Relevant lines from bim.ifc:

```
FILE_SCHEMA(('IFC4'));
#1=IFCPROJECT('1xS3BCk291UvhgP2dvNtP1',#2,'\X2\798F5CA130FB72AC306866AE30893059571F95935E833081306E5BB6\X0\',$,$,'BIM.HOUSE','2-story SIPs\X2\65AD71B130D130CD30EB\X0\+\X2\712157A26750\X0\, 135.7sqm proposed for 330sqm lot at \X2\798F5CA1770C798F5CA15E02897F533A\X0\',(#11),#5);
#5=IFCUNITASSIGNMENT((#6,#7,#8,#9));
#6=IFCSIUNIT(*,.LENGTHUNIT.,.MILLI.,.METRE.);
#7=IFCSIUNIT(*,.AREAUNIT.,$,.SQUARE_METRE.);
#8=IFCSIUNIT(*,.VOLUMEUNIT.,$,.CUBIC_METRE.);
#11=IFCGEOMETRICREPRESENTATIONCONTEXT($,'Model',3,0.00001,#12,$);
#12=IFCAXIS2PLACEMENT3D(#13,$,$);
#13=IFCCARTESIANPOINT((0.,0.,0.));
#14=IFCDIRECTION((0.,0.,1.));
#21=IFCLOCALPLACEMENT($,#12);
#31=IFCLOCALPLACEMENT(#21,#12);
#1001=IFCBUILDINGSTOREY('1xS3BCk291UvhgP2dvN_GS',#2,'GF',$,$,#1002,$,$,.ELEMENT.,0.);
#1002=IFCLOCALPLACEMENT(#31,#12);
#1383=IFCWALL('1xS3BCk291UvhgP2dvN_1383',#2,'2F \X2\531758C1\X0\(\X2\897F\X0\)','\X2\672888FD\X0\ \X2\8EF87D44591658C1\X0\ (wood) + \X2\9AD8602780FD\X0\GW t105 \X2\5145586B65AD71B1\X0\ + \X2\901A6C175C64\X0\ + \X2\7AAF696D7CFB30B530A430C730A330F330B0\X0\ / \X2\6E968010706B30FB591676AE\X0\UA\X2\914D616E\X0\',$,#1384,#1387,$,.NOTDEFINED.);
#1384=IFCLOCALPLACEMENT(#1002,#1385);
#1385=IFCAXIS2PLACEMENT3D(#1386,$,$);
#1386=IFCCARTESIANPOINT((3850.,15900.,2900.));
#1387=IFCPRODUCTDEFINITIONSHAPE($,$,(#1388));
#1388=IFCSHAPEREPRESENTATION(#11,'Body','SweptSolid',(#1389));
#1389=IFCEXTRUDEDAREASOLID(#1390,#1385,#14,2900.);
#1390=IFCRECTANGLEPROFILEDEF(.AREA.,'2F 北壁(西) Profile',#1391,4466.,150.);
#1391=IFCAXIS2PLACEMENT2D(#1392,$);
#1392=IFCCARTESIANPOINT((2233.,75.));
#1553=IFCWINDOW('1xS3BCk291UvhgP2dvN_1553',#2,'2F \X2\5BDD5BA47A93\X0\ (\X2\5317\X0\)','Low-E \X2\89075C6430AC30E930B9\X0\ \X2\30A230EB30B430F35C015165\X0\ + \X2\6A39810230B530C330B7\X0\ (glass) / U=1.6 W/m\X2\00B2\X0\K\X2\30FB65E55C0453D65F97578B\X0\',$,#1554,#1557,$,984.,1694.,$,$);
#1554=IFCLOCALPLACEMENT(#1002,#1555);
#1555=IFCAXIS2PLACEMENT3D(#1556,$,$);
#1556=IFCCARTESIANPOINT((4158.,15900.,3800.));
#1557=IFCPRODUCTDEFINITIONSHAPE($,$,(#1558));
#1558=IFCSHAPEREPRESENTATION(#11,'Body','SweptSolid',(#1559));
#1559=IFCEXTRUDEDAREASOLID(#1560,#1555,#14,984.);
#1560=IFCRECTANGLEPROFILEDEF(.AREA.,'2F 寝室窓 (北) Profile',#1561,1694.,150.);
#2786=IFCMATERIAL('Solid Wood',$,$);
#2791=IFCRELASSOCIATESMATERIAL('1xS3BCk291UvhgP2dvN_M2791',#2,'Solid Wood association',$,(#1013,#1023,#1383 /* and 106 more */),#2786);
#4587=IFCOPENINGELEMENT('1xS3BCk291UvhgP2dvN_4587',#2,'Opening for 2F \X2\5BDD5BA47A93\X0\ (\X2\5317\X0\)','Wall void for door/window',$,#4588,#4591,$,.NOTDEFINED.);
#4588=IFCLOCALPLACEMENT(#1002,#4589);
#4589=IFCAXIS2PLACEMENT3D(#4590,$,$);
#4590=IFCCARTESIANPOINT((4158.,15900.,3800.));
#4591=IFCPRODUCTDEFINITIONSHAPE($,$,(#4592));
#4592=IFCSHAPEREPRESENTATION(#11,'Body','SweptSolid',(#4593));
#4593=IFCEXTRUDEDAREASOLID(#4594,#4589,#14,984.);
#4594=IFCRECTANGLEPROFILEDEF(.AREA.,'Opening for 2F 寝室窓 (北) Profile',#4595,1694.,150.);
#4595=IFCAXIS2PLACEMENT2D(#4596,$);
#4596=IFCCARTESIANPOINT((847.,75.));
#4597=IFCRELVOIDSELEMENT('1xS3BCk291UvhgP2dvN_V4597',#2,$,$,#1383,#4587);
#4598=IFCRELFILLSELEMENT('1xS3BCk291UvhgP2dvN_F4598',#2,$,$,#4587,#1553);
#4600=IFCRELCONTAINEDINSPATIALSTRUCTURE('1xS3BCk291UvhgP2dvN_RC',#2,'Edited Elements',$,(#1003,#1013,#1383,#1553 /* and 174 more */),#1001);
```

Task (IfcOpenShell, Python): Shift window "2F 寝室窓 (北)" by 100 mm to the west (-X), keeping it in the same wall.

```python
import ifcopenshell
import ifcopenshell.api.geometry
import ifcopenshell.util.placement
import ifcopenshell.util.unit

model = ifcopenshell.open("bim.ifc")
unit_scale = ifcopenshell.util.unit.calculate_unit_scale(model)

window = model.by_guid("1xS3BCk291UvhgP2dvN_1553")
opening = window.FillsVoids[0].RelatingOpeningElement
wall = opening.VoidsElements[0].RelatingBuildingElement

wall_matrix = ifcopenshell.util.placement.get_local_placement(wall.ObjectPlacement)
shift = wall_matrix[:3, 0] * -0.1 / unit_scale
before = ifcopenshell.util.placement.get_local_placement(window.ObjectPlacement)[:3, 3].copy()

# The window is not placed relative to its opening, so move both.
for product in (opening, window):
    matrix = ifcopenshell.util.placement.get_local_placement(product.ObjectPlacement)
    matrix[:3, 3] += shift
    ifcopenshell.api.geometry.edit_object_placement(model, product=product, matrix=matrix, is_si=False)

after = ifcopenshell.util.placement.get_local_placement(window.ObjectPlacement)[:3, 3]
print("window moved by", (after - before).round(3) + 0.0)

model.write("bim_rev.ifc")
```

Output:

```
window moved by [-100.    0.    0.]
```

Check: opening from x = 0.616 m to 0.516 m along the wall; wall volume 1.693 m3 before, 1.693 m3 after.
